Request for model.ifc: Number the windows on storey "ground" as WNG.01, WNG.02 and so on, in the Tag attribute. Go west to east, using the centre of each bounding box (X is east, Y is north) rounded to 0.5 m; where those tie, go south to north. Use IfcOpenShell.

First a look at what the model holds.

```python
import ifcopenshell
import ifcopenshell.util.element
import ifcopenshell.util.placement

model = ifcopenshell.open("model.ifc")
print(model.schema)
storey = next(s for s in model.by_type("IfcBuildingStorey") if s.Name == "ground")
windows = [e for e in ifcopenshell.util.element.get_decomposition(storey) if e.is_a("IfcWindow")]
for e in sorted(windows, key=lambda e: e.id()):
    origin = ifcopenshell.util.placement.get_local_placement(e.ObjectPlacement)[:3, 3]
    print(e.id(), e.Tag, e.Name, origin.round(2) + 0.0, sep=" | ")
```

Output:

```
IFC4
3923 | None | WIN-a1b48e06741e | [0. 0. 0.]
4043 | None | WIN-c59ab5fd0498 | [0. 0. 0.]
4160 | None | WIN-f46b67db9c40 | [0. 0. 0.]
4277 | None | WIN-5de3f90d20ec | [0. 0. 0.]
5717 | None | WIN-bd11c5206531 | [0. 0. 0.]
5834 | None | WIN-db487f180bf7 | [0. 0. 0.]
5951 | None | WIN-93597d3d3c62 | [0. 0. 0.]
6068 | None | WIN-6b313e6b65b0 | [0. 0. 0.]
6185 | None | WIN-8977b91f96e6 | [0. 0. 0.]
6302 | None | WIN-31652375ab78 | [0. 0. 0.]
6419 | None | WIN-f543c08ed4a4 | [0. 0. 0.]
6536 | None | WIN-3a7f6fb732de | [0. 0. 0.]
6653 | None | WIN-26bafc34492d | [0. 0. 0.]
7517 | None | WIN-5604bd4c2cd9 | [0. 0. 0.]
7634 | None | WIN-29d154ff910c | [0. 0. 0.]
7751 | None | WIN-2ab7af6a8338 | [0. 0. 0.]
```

```python
import ifcopenshell
import ifcopenshell.geom
import ifcopenshell.util.element
import ifcopenshell.util.shape

model = ifcopenshell.open("model.ifc")
settings = ifcopenshell.geom.settings()
settings.set("use-world-coords", True)


def centre(element):
    shape = ifcopenshell.geom.create_shape(settings, element)
    return ifcopenshell.util.shape.get_bbox_centroid(shape.geometry)


storey = next(s for s in model.by_type("IfcBuildingStorey") if s.Name == "ground")
windows = [e for e in ifcopenshell.util.element.get_decomposition(storey) if e.is_a("IfcWindow")]

# Insertion points can sit at a corner or the storey origin, so sort by the geometry (in metres).
centres = {e: centre(e) for e in windows}
windows.sort(key=lambda e: (round(centres[e][0] / 0.5), centres[e][1]))

for i, e in enumerate(windows, start=1):
    number = f"WNG.{i:02d}"
    e.Tag = number
    print(e.id(), number)

model.write("model_edited.ifc")
```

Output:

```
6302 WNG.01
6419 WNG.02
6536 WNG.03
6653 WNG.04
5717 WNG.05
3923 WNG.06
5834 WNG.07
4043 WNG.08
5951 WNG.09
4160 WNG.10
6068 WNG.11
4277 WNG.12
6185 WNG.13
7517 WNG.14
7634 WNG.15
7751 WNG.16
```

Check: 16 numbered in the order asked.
